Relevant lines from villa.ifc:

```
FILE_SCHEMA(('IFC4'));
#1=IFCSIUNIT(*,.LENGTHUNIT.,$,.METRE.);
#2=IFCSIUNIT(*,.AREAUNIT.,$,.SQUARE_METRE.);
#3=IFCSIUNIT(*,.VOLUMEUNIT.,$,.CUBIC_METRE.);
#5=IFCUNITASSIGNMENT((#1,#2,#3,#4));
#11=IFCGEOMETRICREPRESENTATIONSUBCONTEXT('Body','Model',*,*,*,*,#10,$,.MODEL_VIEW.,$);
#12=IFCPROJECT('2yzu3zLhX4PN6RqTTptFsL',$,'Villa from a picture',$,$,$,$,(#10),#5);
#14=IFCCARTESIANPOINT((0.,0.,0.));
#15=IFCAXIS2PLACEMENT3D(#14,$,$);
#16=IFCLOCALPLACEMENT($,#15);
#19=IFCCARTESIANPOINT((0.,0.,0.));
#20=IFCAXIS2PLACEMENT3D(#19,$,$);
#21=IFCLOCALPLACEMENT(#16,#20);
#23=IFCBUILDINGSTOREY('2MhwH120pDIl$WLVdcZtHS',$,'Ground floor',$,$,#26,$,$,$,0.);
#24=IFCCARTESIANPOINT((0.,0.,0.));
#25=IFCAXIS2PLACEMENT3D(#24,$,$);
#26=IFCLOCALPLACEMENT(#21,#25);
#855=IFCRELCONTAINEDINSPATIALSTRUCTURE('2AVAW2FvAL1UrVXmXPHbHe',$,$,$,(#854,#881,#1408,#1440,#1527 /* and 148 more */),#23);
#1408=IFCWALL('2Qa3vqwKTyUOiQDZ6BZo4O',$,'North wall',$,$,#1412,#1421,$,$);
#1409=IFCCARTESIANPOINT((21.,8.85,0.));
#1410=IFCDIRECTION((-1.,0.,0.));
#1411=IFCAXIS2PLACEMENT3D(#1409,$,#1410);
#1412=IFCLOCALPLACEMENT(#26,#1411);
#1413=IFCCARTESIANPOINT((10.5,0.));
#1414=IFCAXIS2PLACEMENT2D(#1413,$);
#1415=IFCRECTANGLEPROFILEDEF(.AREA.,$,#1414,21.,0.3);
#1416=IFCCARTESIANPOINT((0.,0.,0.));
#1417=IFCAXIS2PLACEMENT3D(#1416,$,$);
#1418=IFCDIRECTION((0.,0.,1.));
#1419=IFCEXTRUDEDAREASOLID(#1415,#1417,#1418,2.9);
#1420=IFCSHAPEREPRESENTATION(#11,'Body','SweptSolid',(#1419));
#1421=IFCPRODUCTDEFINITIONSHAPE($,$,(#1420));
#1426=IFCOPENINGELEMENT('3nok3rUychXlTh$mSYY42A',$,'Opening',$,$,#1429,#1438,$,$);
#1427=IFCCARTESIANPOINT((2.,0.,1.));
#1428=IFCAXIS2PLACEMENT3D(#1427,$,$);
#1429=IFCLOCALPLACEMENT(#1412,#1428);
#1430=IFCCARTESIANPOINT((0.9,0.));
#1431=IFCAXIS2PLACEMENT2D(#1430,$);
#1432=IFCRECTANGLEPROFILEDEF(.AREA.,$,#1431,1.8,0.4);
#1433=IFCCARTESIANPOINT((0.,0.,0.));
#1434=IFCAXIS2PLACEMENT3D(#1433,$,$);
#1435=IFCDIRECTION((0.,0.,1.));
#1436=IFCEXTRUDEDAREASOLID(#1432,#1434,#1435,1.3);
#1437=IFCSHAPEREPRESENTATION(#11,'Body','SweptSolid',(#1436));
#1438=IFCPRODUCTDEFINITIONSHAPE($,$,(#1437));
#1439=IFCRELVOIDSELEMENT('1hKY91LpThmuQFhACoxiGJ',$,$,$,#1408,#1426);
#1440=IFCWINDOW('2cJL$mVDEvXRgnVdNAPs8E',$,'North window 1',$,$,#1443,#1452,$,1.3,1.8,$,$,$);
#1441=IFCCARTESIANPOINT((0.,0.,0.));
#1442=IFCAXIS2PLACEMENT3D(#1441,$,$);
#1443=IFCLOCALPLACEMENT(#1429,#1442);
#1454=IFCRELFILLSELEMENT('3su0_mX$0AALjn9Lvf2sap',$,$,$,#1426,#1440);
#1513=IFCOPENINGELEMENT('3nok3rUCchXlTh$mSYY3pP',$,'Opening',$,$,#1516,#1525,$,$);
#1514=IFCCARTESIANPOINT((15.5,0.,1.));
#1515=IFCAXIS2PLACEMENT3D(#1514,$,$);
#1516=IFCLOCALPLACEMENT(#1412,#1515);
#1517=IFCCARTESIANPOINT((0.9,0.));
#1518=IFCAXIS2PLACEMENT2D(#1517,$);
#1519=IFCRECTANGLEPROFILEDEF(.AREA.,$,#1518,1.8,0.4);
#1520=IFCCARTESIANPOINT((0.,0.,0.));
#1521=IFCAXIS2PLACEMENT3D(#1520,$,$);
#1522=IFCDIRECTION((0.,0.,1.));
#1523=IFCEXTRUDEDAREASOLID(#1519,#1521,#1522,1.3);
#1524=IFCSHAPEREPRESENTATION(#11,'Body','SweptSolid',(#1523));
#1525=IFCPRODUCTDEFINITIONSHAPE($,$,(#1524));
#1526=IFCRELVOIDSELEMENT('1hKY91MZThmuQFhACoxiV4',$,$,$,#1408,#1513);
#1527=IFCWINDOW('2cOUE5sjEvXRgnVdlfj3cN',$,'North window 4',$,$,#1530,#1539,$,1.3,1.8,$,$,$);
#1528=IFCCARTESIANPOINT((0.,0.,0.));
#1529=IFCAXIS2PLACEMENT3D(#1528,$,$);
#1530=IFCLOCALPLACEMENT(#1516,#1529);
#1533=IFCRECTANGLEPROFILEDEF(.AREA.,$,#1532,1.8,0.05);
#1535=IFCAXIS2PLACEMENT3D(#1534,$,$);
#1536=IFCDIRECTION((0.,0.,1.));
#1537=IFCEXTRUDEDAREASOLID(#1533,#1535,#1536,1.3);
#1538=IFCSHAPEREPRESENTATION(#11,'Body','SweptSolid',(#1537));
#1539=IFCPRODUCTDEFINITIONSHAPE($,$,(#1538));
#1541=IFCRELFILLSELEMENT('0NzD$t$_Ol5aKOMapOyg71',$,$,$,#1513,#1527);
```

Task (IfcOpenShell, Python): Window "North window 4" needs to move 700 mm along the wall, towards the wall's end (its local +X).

```python
import ifcopenshell
import ifcopenshell.api.geometry
import ifcopenshell.util.placement

model = ifcopenshell.open("villa.ifc")

window = model.by_guid("2cOUE5sjEvXRgnVdlfj3cN")
opening = window.FillsVoids[0].RelatingOpeningElement
wall = opening.VoidsElements[0].RelatingBuildingElement

wall_matrix = ifcopenshell.util.placement.get_local_placement(wall.ObjectPlacement)
shift = wall_matrix[:3, 0] * 0.7
before = ifcopenshell.util.placement.get_local_placement(window.ObjectPlacement)[:3, 3].copy()

# The window is placed relative to its opening, so it follows when the opening moves.
matrix = ifcopenshell.util.placement.get_local_placement(opening.ObjectPlacement)
matrix[:3, 3] += shift
ifcopenshell.api.geometry.edit_object_placement(
    model, product=opening, matrix=matrix, is_si=False, should_transform_children=True
)

after = ifcopenshell.util.placement.get_local_placement(window.ObjectPlacement)[:3, 3]
print("window moved by", (after - before).round(3) + 0.0)

model.write("villa-out.ifc")
```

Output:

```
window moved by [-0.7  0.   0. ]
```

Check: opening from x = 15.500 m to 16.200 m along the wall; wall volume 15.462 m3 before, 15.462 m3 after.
